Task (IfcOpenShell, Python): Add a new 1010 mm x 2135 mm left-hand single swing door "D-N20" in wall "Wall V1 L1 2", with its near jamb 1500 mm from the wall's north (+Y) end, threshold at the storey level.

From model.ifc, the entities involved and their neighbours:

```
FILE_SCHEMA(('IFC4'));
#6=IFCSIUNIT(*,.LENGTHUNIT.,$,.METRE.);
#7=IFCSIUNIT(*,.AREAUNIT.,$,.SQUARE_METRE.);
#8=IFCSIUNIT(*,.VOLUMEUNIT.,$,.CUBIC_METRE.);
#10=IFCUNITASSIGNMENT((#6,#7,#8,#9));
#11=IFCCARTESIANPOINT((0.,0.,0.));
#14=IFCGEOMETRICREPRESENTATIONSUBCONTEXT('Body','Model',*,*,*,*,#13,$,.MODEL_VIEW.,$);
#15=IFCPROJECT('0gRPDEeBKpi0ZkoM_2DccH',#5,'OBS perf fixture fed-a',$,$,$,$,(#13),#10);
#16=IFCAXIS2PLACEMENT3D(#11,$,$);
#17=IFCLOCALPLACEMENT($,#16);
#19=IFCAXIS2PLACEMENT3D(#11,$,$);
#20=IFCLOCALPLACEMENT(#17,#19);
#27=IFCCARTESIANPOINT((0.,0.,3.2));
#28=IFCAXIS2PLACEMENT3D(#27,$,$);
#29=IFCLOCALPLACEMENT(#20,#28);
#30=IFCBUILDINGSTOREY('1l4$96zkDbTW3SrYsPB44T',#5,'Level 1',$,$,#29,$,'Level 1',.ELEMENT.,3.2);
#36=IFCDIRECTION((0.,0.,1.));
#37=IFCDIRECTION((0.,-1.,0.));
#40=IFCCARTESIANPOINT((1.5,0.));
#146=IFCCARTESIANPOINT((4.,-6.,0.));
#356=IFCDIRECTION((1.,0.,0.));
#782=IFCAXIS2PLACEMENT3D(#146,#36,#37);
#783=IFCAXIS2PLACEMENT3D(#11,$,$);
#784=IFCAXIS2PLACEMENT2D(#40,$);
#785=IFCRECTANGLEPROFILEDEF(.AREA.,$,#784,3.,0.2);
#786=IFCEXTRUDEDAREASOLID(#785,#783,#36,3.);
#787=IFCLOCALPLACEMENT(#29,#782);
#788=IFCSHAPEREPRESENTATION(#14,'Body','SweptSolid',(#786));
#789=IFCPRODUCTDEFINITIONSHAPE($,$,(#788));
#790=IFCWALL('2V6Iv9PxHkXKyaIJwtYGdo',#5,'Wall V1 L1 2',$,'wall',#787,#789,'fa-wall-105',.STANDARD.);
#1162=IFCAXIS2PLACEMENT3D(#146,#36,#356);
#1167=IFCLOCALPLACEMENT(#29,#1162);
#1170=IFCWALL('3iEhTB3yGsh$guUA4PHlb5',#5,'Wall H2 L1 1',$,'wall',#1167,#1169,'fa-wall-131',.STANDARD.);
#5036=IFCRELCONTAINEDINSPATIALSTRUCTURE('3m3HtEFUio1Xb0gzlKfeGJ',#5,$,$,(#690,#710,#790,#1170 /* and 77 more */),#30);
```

```python
import numpy as np
import ifcopenshell
import ifcopenshell.api.feature
import ifcopenshell.api.geometry
import ifcopenshell.api.root
import ifcopenshell.api.spatial
import ifcopenshell.geom
import ifcopenshell.util.element
import ifcopenshell.util.placement
import ifcopenshell.util.representation
import ifcopenshell.util.shape
import ifcopenshell.util.unit

model = ifcopenshell.open("model.ifc")
unit_scale = ifcopenshell.util.unit.calculate_unit_scale(model)
settings = ifcopenshell.geom.settings()


def volume(element):
    """Net volume in cubic metres, openings subtracted."""
    shape = ifcopenshell.geom.create_shape(settings, element)
    return ifcopenshell.util.shape.get_volume(shape.geometry)


wall = model.by_guid("2V6Iv9PxHkXKyaIJwtYGdo")
storey = ifcopenshell.util.element.get_container(wall, ifc_class="IfcBuildingStorey")
context = ifcopenshell.util.representation.get_context(model, "Model", "Body", "MODEL_VIEW")
before = volume(wall)

width, height, from_end, sill = 1.01, 2.135, 1.5, 0.0  # metres

# The wall runs along its own X axis, and the end named is its -X end.
wall_shape = ifcopenshell.geom.create_shape(settings, wall)
x, y, z = ifcopenshell.util.shape.get_vertices(wall_shape.geometry).T
start = x.min() + from_end
face, thickness = float(y.min()), float(y.max() - y.min())
wall_matrix = ifcopenshell.util.placement.get_local_placement(wall.ObjectPlacement)
level = ifcopenshell.util.placement.get_local_placement(storey.ObjectPlacement)[2, 3]


def in_wall(x, y):
    """Placement at x, y metres in the wall's axes, at sill height."""
    matrix = wall_matrix.copy()
    matrix[:, 3] = wall_matrix @ np.array([x / unit_scale, y / unit_scale, 0.0, 1.0])
    matrix[2, 3] = level + sill / unit_scale
    return matrix


# Opening: a box that overshoots both wall faces by 50 mm.
opening = ifcopenshell.api.root.create_entity(model, ifc_class="IfcOpeningElement", predefined_type="OPENING")
box = ifcopenshell.api.geometry.add_wall_representation(
    model, context=context, length=width, height=height, thickness=thickness + 0.1
)
ifcopenshell.api.geometry.assign_representation(model, product=opening, representation=box)
ifcopenshell.api.geometry.edit_object_placement(model, product=opening, matrix=in_wall(start, face - 0.05), is_si=False)
ifcopenshell.api.feature.add_feature(model, feature=opening, element=wall)

door = ifcopenshell.api.root.create_entity(model, ifc_class="IfcDoor", name="D-N20", predefined_type="DOOR")
door.OverallWidth, door.OverallHeight = width / unit_scale, height / unit_scale
door.OperationType = "SINGLE_SWING_LEFT"
body = ifcopenshell.api.geometry.add_door_representation(
    model,
    context=context,
    overall_width=door.OverallWidth,
    overall_height=door.OverallHeight,
    operation_type="SINGLE_SWING_LEFT",
    lining_properties={"LiningDepth": thickness / unit_scale, "ThresholdDepth": thickness / unit_scale},
)
ifcopenshell.api.geometry.assign_representation(model, product=door, representation=body)
ifcopenshell.api.spatial.assign_container(model, products=[door], relating_structure=storey)
ifcopenshell.api.feature.add_filling(model, opening=opening, element=door)

# The lining spans the wall, so the door starts at the wall face.
ifcopenshell.api.geometry.edit_object_placement(model, product=door, matrix=in_wall(start, face), is_si=False)

after = volume(wall)

print(f"wall volume {before:.3f} -> {after:.3f} m3")

model.write("model-out.ifc")
```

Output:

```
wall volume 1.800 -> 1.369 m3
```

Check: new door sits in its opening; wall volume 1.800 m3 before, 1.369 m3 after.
